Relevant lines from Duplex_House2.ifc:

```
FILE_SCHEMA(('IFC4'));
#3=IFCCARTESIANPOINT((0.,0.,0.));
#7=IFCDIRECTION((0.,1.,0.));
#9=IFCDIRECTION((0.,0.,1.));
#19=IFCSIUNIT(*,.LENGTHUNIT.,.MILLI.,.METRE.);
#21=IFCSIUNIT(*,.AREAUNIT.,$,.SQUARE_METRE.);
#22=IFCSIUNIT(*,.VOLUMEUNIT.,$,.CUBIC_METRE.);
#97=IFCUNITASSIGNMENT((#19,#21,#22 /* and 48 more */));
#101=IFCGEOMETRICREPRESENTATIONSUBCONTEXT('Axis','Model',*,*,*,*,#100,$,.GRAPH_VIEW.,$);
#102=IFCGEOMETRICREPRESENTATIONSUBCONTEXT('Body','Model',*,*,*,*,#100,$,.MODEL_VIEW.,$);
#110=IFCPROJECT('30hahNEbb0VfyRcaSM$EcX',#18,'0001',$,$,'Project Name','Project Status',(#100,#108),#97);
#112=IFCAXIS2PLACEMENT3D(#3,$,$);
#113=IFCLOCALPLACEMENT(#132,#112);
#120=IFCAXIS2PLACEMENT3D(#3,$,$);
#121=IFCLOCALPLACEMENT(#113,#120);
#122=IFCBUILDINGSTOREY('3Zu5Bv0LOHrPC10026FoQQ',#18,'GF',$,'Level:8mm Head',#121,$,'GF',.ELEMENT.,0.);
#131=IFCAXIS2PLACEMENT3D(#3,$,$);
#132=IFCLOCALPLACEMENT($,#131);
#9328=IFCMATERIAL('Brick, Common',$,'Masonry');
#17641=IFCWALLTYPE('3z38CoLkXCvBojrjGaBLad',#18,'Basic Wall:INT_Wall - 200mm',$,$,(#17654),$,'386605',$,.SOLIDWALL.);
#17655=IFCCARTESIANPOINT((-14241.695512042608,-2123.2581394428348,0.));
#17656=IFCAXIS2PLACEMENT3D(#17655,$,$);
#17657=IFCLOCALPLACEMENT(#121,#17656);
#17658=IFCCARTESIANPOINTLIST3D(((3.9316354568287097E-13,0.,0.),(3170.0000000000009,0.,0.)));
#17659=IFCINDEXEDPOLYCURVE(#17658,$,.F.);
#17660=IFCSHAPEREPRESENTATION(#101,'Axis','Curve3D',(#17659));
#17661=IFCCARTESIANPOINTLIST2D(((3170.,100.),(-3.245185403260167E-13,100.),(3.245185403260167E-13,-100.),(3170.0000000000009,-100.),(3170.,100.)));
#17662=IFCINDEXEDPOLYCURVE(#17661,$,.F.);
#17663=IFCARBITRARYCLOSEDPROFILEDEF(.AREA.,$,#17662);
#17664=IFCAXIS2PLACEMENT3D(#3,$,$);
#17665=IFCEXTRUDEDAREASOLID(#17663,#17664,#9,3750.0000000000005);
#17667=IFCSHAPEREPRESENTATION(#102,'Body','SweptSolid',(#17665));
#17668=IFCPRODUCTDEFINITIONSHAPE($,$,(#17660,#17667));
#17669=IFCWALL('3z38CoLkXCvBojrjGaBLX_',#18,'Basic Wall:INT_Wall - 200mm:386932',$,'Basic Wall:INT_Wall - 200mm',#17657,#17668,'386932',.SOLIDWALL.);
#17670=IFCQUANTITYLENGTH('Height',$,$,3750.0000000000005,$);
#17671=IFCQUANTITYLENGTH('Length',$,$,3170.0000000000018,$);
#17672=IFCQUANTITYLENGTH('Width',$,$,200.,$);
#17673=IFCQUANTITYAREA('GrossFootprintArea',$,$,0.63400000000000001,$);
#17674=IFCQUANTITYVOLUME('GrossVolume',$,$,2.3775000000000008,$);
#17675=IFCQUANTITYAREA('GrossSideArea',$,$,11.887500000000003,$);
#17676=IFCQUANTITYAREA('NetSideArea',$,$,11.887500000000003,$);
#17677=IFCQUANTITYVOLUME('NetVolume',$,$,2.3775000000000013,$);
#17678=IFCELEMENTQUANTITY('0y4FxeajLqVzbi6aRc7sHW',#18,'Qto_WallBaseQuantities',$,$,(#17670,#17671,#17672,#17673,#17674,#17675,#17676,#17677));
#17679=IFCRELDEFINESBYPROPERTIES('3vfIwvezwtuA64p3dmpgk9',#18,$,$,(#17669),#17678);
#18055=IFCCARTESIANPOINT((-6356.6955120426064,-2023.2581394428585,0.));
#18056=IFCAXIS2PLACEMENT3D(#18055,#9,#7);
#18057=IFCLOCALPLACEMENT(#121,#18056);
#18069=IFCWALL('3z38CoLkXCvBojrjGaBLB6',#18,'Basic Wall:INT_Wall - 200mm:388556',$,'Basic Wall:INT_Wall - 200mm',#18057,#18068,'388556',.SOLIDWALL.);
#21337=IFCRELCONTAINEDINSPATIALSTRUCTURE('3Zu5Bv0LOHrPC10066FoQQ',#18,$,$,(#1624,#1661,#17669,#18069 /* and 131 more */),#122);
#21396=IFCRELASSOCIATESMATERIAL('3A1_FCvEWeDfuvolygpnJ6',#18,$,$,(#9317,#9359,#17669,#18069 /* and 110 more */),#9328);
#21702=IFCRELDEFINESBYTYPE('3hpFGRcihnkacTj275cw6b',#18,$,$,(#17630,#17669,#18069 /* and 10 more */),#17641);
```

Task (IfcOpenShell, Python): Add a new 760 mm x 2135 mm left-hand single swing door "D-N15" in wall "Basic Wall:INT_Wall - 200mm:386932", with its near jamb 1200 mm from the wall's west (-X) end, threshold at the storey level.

```python
import numpy as np
import ifcopenshell
import ifcopenshell.api.feature
import ifcopenshell.api.geometry
import ifcopenshell.api.pset
import ifcopenshell.api.root
import ifcopenshell.api.spatial
import ifcopenshell.geom
import ifcopenshell.util.element
import ifcopenshell.util.placement
import ifcopenshell.util.representation
import ifcopenshell.util.shape
import ifcopenshell.util.unit

model = ifcopenshell.open("Duplex_House2.ifc")
unit_scale = ifcopenshell.util.unit.calculate_unit_scale(model)
area_scale = ifcopenshell.util.unit.calculate_unit_scale(model, "AREAUNIT")
volume_scale = ifcopenshell.util.unit.calculate_unit_scale(model, "VOLUMEUNIT")
settings = ifcopenshell.geom.settings()


def volume(element):
    """Net volume in cubic metres, openings subtracted."""
    shape = ifcopenshell.geom.create_shape(settings, element)
    return ifcopenshell.util.shape.get_volume(shape.geometry)


wall = model.by_guid("3z38CoLkXCvBojrjGaBLX_")
storey = ifcopenshell.util.element.get_container(wall, ifc_class="IfcBuildingStorey")
context = ifcopenshell.util.representation.get_context(model, "Model", "Body", "MODEL_VIEW")
before = volume(wall)

width, height, from_end, sill = 0.76, 2.135, 1.2, 0.0  # metres

# The wall runs along its own X axis, and the end named is its -X end.
wall_shape = ifcopenshell.geom.create_shape(settings, wall)
x, y, z = ifcopenshell.util.shape.get_vertices(wall_shape.geometry).T
start = x.min() + from_end
face, thickness = float(y.min()), float(y.max() - y.min())
wall_matrix = ifcopenshell.util.placement.get_local_placement(wall.ObjectPlacement)
level = ifcopenshell.util.placement.get_local_placement(storey.ObjectPlacement)[2, 3]


def in_wall(x, y):
    """Placement at x, y metres in the wall's axes, at sill height."""
    matrix = wall_matrix.copy()
    matrix[:, 3] = wall_matrix @ np.array([x / unit_scale, y / unit_scale, 0.0, 1.0])
    matrix[2, 3] = level + sill / unit_scale
    return matrix


# Opening: a box that overshoots both wall faces by 50 mm.
opening = ifcopenshell.api.root.create_entity(model, ifc_class="IfcOpeningElement", predefined_type="OPENING")
box = ifcopenshell.api.geometry.add_wall_representation(
    model, context=context, length=width, height=height, thickness=thickness + 0.1
)
ifcopenshell.api.geometry.assign_representation(model, product=opening, representation=box)
ifcopenshell.api.geometry.edit_object_placement(model, product=opening, matrix=in_wall(start, face - 0.05), is_si=False)
ifcopenshell.api.feature.add_feature(model, feature=opening, element=wall)

door = ifcopenshell.api.root.create_entity(model, ifc_class="IfcDoor", name="D-N15", predefined_type="DOOR")
door.OverallWidth, door.OverallHeight = width / unit_scale, height / unit_scale
door.OperationType = "SINGLE_SWING_LEFT"
body = ifcopenshell.api.geometry.add_door_representation(
    model,
    context=context,
    overall_width=door.OverallWidth,
    overall_height=door.OverallHeight,
    operation_type="SINGLE_SWING_LEFT",
    lining_properties={"LiningDepth": thickness / unit_scale, "ThresholdDepth": thickness / unit_scale},
)
ifcopenshell.api.geometry.assign_representation(model, product=door, representation=body)
ifcopenshell.api.spatial.assign_container(model, products=[door], relating_structure=storey)
ifcopenshell.api.feature.add_filling(model, opening=opening, element=door)

# The lining spans the wall, so the door starts at the wall face.
ifcopenshell.api.geometry.edit_object_placement(model, product=door, matrix=in_wall(start, face), is_si=False)

after = volume(wall)

# Update the wall's stored quantities.
qto = model.by_id(ifcopenshell.util.element.get_pset(wall, "Qto_WallBaseQuantities", should_inherit=False)["id"])
ifcopenshell.api.pset.edit_qto(model, qto=qto, properties={
    "NetSideArea": after / thickness / area_scale,
    "NetVolume": after / volume_scale,
})

print(f"wall volume {before:.3f} -> {after:.3f} m3")

model.write("Duplex_House2-out.ifc")
```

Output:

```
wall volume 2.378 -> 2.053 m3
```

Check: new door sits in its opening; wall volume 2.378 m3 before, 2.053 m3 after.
